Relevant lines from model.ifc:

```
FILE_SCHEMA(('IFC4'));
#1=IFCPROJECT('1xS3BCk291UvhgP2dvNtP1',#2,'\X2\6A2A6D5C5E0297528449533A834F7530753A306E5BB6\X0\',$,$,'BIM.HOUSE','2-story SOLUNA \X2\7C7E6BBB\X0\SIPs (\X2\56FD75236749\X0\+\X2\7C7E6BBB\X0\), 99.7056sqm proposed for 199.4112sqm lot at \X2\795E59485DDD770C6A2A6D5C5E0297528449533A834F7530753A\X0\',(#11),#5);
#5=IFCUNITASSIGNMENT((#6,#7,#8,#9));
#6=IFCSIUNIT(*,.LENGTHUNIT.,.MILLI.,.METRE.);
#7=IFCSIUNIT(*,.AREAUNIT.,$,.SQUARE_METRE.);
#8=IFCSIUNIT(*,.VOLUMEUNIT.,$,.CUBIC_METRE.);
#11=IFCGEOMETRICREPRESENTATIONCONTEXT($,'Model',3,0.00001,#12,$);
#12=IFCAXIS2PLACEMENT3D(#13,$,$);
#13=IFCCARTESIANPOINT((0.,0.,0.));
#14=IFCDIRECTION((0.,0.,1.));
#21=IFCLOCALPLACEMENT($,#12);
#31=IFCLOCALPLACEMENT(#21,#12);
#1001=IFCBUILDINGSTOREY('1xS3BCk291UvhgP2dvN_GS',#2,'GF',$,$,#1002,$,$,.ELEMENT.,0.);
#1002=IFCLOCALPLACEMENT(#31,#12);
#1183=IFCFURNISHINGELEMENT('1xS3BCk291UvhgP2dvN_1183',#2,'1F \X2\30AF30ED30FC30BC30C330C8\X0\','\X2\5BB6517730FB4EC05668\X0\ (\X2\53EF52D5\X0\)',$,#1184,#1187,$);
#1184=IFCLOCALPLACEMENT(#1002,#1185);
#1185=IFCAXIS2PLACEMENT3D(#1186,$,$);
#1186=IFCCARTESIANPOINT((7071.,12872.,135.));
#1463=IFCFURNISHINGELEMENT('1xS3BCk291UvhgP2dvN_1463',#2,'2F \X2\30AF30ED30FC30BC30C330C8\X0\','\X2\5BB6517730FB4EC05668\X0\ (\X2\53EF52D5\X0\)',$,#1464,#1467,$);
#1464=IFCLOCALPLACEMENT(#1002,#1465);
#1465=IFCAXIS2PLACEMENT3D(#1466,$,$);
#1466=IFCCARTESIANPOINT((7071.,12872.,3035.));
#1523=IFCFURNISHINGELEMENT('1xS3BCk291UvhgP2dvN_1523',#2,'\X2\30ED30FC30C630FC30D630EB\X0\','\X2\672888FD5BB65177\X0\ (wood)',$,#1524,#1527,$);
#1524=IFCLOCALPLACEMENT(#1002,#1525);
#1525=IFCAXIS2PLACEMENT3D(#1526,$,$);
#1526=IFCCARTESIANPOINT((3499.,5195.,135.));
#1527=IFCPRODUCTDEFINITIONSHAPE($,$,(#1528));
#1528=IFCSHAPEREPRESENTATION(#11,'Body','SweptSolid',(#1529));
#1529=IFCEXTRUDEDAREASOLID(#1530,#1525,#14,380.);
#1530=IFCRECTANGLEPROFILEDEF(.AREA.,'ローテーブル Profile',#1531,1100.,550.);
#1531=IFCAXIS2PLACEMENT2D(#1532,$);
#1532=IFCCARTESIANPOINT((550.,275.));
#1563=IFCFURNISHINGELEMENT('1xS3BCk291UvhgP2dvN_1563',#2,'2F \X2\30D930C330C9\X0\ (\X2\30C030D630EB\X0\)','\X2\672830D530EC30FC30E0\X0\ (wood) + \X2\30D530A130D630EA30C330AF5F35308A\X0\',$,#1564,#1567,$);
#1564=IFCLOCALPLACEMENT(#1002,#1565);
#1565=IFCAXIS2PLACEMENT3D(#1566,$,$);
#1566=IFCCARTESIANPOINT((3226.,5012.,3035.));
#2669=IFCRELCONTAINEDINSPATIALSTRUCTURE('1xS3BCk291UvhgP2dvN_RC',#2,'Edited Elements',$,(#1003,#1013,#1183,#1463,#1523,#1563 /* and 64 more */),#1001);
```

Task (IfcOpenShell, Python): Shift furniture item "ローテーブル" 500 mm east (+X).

```python
import ifcopenshell
import ifcopenshell.api.geometry
import ifcopenshell.util.placement
import ifcopenshell.util.unit

model = ifcopenshell.open("model.ifc")
unit_scale = ifcopenshell.util.unit.calculate_unit_scale(model)

item = model.by_id(1523)
matrix = ifcopenshell.util.placement.get_local_placement(item.ObjectPlacement)
matrix[0, 3] += 0.5 / unit_scale
ifcopenshell.api.geometry.edit_object_placement(model, product=item, matrix=matrix, is_si=False)

print(ifcopenshell.util.placement.get_local_placement(item.ObjectPlacement).round(3) + 0.0)

model.write("model-out.ifc")
```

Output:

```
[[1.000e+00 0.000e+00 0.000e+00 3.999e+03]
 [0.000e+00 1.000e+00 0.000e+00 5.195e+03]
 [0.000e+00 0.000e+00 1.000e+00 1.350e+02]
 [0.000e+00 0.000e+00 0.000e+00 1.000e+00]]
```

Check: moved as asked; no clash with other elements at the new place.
